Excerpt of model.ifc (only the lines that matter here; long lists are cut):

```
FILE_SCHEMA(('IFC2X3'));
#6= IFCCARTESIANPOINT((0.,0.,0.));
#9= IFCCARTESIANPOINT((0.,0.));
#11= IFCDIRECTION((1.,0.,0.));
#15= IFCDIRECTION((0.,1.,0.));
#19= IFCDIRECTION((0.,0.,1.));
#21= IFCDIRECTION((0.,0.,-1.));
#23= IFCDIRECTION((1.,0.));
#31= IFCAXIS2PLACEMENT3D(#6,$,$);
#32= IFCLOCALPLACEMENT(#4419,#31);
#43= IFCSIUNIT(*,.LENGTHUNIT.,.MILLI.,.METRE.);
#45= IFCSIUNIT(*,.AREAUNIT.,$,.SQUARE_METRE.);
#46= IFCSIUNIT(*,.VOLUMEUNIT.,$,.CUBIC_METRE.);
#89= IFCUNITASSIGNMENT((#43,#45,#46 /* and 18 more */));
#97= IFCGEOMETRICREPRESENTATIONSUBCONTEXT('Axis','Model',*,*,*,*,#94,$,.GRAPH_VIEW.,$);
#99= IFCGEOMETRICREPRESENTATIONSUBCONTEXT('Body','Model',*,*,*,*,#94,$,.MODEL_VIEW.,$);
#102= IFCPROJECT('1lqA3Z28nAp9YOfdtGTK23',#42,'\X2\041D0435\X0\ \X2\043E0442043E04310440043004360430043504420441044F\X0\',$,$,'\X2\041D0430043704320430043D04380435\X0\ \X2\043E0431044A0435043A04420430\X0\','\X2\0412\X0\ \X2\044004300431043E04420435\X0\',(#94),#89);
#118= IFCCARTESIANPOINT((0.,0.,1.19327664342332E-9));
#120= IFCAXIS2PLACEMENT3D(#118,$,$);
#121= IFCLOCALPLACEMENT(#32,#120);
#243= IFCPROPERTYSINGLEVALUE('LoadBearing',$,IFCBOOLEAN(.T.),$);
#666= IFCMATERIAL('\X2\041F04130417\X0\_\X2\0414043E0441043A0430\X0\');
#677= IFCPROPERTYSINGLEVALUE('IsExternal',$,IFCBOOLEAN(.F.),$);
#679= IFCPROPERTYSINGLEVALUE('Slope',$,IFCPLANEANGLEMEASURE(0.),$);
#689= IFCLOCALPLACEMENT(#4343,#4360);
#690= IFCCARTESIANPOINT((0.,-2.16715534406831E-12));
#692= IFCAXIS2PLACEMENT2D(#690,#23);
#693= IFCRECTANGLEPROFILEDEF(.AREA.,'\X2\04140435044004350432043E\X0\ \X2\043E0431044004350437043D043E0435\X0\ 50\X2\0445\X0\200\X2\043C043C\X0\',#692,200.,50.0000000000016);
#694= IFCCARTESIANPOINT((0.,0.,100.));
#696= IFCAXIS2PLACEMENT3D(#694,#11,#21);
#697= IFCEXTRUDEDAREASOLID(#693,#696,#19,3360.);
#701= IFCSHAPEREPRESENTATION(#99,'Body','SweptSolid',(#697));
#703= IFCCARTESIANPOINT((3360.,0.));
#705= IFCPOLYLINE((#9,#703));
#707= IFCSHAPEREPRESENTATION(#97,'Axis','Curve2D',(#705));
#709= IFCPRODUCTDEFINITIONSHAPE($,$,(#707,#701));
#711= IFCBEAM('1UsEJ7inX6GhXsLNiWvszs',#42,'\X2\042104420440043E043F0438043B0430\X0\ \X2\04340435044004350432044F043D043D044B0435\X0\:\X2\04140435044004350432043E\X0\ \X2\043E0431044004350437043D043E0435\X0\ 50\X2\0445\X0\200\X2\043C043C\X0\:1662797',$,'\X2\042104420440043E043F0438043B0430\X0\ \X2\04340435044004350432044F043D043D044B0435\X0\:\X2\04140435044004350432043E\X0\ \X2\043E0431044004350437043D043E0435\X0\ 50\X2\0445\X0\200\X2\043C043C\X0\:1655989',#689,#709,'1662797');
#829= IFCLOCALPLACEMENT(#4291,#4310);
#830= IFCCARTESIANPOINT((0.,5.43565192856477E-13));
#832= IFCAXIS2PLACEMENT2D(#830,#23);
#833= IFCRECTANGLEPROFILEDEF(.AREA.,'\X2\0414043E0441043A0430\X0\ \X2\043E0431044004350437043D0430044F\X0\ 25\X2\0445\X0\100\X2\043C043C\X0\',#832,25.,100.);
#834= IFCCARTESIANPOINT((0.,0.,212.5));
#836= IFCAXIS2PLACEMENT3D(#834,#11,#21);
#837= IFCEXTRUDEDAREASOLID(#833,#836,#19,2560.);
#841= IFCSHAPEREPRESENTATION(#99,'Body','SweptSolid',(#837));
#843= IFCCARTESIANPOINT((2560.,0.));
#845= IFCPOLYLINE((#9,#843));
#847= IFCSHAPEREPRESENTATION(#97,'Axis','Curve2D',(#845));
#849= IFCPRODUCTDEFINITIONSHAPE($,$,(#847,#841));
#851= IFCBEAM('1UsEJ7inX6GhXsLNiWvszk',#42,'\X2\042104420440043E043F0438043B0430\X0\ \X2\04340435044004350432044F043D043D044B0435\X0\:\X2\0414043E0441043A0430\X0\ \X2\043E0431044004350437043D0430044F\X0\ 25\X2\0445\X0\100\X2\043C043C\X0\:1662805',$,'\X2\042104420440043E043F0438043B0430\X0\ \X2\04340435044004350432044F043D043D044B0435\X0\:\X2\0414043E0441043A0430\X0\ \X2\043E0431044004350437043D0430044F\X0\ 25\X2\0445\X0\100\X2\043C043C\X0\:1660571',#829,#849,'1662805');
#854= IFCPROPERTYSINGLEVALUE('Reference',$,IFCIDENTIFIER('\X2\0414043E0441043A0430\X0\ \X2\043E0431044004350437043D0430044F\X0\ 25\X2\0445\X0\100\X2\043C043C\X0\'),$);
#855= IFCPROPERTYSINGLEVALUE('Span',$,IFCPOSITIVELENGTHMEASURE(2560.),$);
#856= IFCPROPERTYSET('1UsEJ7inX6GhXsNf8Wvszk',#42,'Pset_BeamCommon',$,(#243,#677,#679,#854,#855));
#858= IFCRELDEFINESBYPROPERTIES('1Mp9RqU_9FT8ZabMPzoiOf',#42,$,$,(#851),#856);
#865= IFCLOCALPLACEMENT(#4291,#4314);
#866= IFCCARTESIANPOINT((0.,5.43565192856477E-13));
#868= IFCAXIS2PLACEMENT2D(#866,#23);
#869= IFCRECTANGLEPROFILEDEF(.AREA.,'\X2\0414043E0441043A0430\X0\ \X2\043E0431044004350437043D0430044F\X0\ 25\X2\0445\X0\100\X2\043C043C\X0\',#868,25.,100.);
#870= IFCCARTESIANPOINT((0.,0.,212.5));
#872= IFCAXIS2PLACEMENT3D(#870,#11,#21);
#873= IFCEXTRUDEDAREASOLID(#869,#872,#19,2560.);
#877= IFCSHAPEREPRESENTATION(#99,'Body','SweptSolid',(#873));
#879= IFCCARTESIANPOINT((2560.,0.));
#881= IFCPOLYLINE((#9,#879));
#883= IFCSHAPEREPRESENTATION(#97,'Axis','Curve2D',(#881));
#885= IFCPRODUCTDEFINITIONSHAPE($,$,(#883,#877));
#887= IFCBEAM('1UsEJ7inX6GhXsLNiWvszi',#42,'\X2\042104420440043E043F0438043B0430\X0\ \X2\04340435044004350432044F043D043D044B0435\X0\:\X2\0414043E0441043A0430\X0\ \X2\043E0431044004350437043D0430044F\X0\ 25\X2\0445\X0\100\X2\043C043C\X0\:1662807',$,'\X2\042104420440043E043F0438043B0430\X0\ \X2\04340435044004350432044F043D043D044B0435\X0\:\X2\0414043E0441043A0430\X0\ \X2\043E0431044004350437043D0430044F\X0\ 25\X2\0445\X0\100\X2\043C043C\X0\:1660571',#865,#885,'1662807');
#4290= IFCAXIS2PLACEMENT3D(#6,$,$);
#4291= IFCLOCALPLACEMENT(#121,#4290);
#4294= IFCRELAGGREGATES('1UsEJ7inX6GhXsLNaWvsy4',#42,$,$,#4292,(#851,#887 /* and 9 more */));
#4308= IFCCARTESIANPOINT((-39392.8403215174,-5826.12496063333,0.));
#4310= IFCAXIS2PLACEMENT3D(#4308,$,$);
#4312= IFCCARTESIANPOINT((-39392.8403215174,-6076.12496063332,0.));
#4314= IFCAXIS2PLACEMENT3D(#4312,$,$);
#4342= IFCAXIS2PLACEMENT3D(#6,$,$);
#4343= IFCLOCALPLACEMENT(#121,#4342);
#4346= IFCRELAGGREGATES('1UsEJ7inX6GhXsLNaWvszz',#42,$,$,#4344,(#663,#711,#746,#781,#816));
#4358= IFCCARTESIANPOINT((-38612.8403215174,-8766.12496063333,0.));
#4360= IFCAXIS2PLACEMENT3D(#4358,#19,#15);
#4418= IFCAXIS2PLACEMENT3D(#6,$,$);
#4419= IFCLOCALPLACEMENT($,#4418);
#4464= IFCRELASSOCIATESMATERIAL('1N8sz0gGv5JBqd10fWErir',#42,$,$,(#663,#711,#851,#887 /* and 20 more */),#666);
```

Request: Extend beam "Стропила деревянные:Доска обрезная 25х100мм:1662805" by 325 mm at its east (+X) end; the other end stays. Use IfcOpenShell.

```python
import numpy as np
import ifcopenshell
import ifcopenshell.api.pset
import ifcopenshell.util.element
import ifcopenshell.util.representation
import ifcopenshell.util.unit

model = ifcopenshell.open("model.ifc")
unit_scale = ifcopenshell.util.unit.calculate_unit_scale(model)

member = model.by_guid("1UsEJ7inX6GhXsLNiWvszk")
change = 0.325 / unit_scale

# The extrusion runs towards the end named, so only its depth changes.
body = ifcopenshell.util.representation.get_representation(member, "Model", "Body")
solid = body.Items[0]
old_length = solid.Depth
solid.Depth += change

# Move the axis end point with it.
axis = next(r for r in member.Representation.Representations if r.RepresentationIdentifier == "Axis").Items[0]
start, end = (np.array(p.Coordinates) for p in axis.Points)
end = end + (end - start) / np.linalg.norm(end - start) * change
point = model.createIfcCartesianPoint(end.tolist())
axis.Points = [axis.Points[0], point]

# Update the stored length and volume.
pset = model.by_id(ifcopenshell.util.element.get_pset(member, "Pset_BeamCommon", should_inherit=False)["id"])
ifcopenshell.api.pset.edit_pset(model, pset=pset, properties={
    "Span": model.create_entity("IfcPositiveLengthMeasure", solid.Depth),
})

print(f"length {old_length:g} -> {solid.Depth:g}")

model.write("model_updated.ifc")
```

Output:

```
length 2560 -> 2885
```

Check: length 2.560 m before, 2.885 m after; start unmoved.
